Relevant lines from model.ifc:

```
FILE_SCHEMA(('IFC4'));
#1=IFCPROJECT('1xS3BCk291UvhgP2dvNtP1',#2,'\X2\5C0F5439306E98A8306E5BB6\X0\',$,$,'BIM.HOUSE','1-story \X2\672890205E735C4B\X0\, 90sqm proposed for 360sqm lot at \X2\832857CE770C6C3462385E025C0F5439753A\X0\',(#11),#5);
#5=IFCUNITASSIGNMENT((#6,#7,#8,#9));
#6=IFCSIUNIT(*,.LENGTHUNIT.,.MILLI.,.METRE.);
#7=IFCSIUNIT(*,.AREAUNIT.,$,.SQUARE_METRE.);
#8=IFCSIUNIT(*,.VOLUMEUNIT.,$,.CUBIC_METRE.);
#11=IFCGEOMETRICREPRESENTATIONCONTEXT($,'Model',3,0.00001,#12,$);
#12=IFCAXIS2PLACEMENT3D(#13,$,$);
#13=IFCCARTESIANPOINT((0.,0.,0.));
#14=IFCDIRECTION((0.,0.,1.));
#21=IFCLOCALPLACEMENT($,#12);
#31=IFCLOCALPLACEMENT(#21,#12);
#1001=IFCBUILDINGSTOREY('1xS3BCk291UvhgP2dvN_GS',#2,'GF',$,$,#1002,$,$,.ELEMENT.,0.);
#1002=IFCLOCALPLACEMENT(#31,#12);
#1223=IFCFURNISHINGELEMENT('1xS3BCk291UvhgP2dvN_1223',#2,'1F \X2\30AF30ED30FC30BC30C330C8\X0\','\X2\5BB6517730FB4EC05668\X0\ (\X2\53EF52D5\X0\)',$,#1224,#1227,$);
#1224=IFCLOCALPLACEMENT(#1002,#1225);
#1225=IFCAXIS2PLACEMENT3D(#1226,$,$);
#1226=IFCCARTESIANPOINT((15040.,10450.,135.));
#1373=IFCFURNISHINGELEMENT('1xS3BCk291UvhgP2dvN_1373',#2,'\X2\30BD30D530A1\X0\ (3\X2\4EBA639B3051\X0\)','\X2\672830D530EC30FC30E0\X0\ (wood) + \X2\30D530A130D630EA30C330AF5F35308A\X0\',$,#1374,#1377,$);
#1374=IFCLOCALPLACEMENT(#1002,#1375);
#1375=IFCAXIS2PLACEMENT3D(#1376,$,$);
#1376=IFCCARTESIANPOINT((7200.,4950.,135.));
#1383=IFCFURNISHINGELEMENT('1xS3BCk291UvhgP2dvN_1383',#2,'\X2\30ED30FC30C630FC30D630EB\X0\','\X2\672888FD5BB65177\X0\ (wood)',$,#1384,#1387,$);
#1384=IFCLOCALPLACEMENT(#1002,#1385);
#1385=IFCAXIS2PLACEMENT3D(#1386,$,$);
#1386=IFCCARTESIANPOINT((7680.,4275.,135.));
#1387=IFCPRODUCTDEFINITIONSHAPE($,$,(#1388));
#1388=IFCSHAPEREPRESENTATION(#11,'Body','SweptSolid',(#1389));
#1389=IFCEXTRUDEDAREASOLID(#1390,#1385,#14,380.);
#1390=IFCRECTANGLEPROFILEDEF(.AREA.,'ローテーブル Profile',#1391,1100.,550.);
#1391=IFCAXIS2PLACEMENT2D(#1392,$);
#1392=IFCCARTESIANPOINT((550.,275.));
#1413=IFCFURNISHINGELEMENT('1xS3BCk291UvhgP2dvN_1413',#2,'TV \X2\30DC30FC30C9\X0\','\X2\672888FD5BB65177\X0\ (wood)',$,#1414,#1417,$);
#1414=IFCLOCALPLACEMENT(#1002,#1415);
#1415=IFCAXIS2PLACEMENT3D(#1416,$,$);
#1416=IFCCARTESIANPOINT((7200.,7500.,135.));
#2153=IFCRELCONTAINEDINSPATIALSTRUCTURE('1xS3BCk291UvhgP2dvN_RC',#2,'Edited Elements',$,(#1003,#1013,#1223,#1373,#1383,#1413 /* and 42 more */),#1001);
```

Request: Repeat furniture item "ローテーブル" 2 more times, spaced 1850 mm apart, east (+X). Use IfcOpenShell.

```python
import numpy as np
import ifcopenshell
import ifcopenshell.api.geometry
import ifcopenshell.api.root
import ifcopenshell.util.element
import ifcopenshell.util.placement
import ifcopenshell.util.unit

model = ifcopenshell.open("model.ifc")
unit_scale = ifcopenshell.util.unit.calculate_unit_scale(model)


def reuse_history(source, copy):
    """copy_class also copies each property set's owner history, people and application; keep the originals."""
    for rel in copy.IsDefinedBy:
        if rel.is_a("IfcRelDefinesByProperties") and (history := rel.RelatingPropertyDefinition.OwnerHistory):
            rel.RelatingPropertyDefinition.OwnerHistory = source.OwnerHistory
            ifcopenshell.util.element.remove_deep2(model, history)


source = model.by_id(1383)
base = ifcopenshell.util.placement.get_local_placement(source.ObjectPlacement)
step = np.array([1.0, 0.0, 0.0]) * 1.85 / unit_scale

for i in range(1, 3):
    copy = ifcopenshell.api.root.copy_class(model, product=source)
    copy.Representation = ifcopenshell.util.element.copy_deep(
        model, source.Representation, exclude=["IfcGeometricRepresentationContext", "IfcRepresentationMap"]
    )
    reuse_history(source, copy)
    matrix = base.copy()
    matrix[:3, 3] += i * step
    print("added at", matrix[:3, 3].round(3) + 0.0)
    ifcopenshell.api.geometry.edit_object_placement(model, product=copy, matrix=matrix, is_si=False)

model.write("model_edited.ifc")
```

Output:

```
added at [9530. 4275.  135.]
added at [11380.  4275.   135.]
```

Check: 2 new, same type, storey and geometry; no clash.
